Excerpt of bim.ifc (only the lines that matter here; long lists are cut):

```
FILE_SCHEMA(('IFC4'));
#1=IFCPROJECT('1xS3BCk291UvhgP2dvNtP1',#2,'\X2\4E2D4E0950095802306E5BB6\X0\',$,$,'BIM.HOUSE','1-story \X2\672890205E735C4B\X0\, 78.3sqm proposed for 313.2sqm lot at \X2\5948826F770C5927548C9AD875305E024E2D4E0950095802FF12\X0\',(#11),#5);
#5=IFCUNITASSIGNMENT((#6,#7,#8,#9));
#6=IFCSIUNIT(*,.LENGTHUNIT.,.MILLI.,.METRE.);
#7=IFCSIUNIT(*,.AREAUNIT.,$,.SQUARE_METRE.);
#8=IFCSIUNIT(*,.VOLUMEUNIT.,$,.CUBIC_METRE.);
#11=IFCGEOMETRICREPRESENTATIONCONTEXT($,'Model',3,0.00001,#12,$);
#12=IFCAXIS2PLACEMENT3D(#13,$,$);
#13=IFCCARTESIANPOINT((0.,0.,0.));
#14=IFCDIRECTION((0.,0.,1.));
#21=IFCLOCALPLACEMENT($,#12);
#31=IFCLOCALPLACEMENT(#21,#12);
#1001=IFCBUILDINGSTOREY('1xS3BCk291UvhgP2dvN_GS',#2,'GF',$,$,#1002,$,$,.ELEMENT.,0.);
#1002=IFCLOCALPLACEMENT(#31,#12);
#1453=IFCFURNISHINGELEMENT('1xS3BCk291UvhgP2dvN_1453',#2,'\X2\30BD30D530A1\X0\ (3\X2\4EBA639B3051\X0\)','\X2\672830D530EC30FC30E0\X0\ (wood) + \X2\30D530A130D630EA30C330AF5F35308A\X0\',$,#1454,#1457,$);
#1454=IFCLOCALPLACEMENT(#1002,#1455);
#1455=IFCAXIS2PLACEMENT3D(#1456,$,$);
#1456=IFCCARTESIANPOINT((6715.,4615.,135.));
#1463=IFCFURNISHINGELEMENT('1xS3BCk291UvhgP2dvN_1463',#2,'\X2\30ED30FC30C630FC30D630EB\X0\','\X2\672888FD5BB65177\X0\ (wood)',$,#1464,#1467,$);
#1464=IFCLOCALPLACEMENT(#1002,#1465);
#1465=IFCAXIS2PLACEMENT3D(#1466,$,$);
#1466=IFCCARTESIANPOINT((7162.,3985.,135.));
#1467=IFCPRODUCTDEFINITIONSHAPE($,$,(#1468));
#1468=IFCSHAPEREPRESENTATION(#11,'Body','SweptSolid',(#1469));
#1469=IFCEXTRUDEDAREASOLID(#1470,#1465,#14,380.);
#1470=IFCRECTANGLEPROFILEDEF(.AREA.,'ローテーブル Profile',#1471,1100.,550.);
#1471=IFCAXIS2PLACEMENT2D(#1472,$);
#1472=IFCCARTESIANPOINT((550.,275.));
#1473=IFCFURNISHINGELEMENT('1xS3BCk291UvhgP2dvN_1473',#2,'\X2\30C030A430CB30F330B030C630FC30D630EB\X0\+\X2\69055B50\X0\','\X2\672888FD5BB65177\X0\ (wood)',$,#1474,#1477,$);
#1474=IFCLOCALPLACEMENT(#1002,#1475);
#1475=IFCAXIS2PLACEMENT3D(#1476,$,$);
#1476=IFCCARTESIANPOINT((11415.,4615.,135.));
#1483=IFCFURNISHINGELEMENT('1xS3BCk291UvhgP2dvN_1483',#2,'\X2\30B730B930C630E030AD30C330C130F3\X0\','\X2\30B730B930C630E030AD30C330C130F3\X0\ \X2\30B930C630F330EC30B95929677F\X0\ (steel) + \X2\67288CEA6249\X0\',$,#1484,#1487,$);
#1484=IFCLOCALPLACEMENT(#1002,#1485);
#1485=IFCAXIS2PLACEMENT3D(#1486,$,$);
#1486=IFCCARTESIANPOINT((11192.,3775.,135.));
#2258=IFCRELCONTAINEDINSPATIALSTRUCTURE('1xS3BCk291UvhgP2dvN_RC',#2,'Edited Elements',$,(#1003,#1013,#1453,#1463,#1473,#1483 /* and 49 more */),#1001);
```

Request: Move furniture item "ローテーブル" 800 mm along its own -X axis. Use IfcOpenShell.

```python
import ifcopenshell
import ifcopenshell.api.geometry
import ifcopenshell.util.placement
import ifcopenshell.util.unit

model = ifcopenshell.open("bim.ifc")
unit_scale = ifcopenshell.util.unit.calculate_unit_scale(model)

item = model.by_id(1463)
matrix = ifcopenshell.util.placement.get_local_placement(item.ObjectPlacement)
matrix[:3, 3] -= matrix[:3, 0] * 0.8 / unit_scale
ifcopenshell.api.geometry.edit_object_placement(model, product=item, matrix=matrix, is_si=False)

print(ifcopenshell.util.placement.get_local_placement(item.ObjectPlacement).round(3) + 0.0)

model.write("bim_updated.ifc")
```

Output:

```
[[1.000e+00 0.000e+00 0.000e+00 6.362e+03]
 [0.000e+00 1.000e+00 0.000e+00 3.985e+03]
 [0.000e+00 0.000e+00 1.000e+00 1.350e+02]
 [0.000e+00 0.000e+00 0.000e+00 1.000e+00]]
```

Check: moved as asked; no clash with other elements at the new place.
